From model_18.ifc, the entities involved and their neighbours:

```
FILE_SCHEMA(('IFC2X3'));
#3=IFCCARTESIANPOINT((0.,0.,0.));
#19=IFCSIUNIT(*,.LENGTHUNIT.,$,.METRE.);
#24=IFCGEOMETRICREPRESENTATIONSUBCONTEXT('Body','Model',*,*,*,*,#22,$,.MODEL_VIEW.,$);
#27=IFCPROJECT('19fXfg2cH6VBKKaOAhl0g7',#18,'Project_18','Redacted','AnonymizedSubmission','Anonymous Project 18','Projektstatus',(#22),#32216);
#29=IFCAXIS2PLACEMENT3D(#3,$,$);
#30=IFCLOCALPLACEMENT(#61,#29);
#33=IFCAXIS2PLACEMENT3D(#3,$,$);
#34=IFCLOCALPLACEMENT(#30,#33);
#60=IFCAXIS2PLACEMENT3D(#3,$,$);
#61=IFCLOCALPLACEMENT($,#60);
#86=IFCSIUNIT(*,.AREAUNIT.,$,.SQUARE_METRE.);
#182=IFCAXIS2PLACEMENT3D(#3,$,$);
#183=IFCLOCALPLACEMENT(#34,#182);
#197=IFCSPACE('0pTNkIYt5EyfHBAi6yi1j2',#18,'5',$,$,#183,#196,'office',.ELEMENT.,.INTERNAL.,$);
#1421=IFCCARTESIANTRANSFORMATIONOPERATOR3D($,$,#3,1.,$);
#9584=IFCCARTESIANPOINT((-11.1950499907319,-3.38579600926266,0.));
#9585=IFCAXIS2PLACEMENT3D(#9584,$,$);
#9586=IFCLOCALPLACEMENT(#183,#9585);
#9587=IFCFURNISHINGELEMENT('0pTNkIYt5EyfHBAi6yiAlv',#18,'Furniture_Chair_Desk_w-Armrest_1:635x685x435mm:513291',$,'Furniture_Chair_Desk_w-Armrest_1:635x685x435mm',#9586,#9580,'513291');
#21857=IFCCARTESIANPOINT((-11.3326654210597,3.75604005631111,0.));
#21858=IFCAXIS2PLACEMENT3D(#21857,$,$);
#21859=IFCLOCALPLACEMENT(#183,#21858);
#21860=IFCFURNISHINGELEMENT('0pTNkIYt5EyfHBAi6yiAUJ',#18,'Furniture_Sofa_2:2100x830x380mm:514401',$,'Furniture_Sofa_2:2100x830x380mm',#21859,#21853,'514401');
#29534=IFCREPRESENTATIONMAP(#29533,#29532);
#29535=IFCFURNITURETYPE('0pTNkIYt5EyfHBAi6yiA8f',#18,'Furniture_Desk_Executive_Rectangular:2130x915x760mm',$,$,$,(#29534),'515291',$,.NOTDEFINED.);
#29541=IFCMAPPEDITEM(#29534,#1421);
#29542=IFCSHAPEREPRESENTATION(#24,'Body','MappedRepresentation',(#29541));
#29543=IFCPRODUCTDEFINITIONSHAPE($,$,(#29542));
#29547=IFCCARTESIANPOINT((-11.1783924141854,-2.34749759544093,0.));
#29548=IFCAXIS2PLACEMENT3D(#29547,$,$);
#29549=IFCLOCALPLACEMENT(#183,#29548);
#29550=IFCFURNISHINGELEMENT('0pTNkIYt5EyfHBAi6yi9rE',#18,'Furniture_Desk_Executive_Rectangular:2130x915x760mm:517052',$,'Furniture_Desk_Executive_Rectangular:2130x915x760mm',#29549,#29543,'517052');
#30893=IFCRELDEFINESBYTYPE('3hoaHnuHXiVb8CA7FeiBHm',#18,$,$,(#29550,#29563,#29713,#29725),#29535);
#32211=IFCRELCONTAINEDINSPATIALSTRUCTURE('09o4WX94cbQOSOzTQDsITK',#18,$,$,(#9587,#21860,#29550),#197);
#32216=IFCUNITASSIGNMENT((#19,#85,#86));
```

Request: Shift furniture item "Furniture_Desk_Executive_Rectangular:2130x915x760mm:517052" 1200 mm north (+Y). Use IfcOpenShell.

```python
import ifcopenshell
import ifcopenshell.api.geometry
import ifcopenshell.util.placement
import ifcopenshell.util.unit

model = ifcopenshell.open("model_18.ifc")
unit_scale = ifcopenshell.util.unit.calculate_unit_scale(model)

item = model.by_guid("0pTNkIYt5EyfHBAi6yi9rE")
matrix = ifcopenshell.util.placement.get_local_placement(item.ObjectPlacement)
matrix[1, 3] += 1.2 / unit_scale
ifcopenshell.api.geometry.edit_object_placement(model, product=item, matrix=matrix, is_si=False)

print(ifcopenshell.util.placement.get_local_placement(item.ObjectPlacement).round(3) + 0.0)

model.write("model_18_rev.ifc")
```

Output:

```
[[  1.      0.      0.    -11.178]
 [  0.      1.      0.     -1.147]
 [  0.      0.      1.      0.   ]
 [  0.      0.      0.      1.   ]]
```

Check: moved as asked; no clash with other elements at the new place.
